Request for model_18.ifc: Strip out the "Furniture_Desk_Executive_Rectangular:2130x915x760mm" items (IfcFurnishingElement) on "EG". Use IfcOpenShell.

First a look at what the model holds.

```python
import ifcopenshell
import ifcopenshell.util.element

model = ifcopenshell.open("model_18.ifc")
print(model.schema)
storey = next(s for s in model.by_type("IfcBuildingStorey") if s.Name == "EG")
furniture = [e for e in ifcopenshell.util.element.get_decomposition(storey) if e.is_a("IfcFurnishingElement")]
seen = {}
for e in furniture:
    element_type = ifcopenshell.util.element.get_type(e)
    name = element_type.Name if element_type not in (None, e) else None
    seen[name] = seen.get(name, 0) + 1
for name, count in sorted(seen.items(), key=str):
    print(count, "x", name)
```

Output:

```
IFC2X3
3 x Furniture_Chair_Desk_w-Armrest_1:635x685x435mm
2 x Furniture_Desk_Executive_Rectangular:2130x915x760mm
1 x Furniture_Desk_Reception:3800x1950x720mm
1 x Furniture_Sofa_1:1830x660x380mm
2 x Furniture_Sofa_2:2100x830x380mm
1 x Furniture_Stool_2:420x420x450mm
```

```python
import ifcopenshell
import ifcopenshell.api.root
import ifcopenshell.util.element

model = ifcopenshell.open("model_18.ifc")

storey = next(s for s in model.by_type("IfcBuildingStorey") if s.Name == "EG")
furniture = [e for e in ifcopenshell.util.element.get_decomposition(storey) if e.is_a("IfcFurnishingElement")]
targets = [e for e in furniture if (t := ifcopenshell.util.element.get_type(e)) not in (None, e) and t.Name == "Furniture_Desk_Executive_Rectangular:2130x915x760mm"]

for e in targets:
    ifcopenshell.api.root.remove_product(model, product=e)
print(len(targets), "removed")

model.write("model_18_updated.ifc")
```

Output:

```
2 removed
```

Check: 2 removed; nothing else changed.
